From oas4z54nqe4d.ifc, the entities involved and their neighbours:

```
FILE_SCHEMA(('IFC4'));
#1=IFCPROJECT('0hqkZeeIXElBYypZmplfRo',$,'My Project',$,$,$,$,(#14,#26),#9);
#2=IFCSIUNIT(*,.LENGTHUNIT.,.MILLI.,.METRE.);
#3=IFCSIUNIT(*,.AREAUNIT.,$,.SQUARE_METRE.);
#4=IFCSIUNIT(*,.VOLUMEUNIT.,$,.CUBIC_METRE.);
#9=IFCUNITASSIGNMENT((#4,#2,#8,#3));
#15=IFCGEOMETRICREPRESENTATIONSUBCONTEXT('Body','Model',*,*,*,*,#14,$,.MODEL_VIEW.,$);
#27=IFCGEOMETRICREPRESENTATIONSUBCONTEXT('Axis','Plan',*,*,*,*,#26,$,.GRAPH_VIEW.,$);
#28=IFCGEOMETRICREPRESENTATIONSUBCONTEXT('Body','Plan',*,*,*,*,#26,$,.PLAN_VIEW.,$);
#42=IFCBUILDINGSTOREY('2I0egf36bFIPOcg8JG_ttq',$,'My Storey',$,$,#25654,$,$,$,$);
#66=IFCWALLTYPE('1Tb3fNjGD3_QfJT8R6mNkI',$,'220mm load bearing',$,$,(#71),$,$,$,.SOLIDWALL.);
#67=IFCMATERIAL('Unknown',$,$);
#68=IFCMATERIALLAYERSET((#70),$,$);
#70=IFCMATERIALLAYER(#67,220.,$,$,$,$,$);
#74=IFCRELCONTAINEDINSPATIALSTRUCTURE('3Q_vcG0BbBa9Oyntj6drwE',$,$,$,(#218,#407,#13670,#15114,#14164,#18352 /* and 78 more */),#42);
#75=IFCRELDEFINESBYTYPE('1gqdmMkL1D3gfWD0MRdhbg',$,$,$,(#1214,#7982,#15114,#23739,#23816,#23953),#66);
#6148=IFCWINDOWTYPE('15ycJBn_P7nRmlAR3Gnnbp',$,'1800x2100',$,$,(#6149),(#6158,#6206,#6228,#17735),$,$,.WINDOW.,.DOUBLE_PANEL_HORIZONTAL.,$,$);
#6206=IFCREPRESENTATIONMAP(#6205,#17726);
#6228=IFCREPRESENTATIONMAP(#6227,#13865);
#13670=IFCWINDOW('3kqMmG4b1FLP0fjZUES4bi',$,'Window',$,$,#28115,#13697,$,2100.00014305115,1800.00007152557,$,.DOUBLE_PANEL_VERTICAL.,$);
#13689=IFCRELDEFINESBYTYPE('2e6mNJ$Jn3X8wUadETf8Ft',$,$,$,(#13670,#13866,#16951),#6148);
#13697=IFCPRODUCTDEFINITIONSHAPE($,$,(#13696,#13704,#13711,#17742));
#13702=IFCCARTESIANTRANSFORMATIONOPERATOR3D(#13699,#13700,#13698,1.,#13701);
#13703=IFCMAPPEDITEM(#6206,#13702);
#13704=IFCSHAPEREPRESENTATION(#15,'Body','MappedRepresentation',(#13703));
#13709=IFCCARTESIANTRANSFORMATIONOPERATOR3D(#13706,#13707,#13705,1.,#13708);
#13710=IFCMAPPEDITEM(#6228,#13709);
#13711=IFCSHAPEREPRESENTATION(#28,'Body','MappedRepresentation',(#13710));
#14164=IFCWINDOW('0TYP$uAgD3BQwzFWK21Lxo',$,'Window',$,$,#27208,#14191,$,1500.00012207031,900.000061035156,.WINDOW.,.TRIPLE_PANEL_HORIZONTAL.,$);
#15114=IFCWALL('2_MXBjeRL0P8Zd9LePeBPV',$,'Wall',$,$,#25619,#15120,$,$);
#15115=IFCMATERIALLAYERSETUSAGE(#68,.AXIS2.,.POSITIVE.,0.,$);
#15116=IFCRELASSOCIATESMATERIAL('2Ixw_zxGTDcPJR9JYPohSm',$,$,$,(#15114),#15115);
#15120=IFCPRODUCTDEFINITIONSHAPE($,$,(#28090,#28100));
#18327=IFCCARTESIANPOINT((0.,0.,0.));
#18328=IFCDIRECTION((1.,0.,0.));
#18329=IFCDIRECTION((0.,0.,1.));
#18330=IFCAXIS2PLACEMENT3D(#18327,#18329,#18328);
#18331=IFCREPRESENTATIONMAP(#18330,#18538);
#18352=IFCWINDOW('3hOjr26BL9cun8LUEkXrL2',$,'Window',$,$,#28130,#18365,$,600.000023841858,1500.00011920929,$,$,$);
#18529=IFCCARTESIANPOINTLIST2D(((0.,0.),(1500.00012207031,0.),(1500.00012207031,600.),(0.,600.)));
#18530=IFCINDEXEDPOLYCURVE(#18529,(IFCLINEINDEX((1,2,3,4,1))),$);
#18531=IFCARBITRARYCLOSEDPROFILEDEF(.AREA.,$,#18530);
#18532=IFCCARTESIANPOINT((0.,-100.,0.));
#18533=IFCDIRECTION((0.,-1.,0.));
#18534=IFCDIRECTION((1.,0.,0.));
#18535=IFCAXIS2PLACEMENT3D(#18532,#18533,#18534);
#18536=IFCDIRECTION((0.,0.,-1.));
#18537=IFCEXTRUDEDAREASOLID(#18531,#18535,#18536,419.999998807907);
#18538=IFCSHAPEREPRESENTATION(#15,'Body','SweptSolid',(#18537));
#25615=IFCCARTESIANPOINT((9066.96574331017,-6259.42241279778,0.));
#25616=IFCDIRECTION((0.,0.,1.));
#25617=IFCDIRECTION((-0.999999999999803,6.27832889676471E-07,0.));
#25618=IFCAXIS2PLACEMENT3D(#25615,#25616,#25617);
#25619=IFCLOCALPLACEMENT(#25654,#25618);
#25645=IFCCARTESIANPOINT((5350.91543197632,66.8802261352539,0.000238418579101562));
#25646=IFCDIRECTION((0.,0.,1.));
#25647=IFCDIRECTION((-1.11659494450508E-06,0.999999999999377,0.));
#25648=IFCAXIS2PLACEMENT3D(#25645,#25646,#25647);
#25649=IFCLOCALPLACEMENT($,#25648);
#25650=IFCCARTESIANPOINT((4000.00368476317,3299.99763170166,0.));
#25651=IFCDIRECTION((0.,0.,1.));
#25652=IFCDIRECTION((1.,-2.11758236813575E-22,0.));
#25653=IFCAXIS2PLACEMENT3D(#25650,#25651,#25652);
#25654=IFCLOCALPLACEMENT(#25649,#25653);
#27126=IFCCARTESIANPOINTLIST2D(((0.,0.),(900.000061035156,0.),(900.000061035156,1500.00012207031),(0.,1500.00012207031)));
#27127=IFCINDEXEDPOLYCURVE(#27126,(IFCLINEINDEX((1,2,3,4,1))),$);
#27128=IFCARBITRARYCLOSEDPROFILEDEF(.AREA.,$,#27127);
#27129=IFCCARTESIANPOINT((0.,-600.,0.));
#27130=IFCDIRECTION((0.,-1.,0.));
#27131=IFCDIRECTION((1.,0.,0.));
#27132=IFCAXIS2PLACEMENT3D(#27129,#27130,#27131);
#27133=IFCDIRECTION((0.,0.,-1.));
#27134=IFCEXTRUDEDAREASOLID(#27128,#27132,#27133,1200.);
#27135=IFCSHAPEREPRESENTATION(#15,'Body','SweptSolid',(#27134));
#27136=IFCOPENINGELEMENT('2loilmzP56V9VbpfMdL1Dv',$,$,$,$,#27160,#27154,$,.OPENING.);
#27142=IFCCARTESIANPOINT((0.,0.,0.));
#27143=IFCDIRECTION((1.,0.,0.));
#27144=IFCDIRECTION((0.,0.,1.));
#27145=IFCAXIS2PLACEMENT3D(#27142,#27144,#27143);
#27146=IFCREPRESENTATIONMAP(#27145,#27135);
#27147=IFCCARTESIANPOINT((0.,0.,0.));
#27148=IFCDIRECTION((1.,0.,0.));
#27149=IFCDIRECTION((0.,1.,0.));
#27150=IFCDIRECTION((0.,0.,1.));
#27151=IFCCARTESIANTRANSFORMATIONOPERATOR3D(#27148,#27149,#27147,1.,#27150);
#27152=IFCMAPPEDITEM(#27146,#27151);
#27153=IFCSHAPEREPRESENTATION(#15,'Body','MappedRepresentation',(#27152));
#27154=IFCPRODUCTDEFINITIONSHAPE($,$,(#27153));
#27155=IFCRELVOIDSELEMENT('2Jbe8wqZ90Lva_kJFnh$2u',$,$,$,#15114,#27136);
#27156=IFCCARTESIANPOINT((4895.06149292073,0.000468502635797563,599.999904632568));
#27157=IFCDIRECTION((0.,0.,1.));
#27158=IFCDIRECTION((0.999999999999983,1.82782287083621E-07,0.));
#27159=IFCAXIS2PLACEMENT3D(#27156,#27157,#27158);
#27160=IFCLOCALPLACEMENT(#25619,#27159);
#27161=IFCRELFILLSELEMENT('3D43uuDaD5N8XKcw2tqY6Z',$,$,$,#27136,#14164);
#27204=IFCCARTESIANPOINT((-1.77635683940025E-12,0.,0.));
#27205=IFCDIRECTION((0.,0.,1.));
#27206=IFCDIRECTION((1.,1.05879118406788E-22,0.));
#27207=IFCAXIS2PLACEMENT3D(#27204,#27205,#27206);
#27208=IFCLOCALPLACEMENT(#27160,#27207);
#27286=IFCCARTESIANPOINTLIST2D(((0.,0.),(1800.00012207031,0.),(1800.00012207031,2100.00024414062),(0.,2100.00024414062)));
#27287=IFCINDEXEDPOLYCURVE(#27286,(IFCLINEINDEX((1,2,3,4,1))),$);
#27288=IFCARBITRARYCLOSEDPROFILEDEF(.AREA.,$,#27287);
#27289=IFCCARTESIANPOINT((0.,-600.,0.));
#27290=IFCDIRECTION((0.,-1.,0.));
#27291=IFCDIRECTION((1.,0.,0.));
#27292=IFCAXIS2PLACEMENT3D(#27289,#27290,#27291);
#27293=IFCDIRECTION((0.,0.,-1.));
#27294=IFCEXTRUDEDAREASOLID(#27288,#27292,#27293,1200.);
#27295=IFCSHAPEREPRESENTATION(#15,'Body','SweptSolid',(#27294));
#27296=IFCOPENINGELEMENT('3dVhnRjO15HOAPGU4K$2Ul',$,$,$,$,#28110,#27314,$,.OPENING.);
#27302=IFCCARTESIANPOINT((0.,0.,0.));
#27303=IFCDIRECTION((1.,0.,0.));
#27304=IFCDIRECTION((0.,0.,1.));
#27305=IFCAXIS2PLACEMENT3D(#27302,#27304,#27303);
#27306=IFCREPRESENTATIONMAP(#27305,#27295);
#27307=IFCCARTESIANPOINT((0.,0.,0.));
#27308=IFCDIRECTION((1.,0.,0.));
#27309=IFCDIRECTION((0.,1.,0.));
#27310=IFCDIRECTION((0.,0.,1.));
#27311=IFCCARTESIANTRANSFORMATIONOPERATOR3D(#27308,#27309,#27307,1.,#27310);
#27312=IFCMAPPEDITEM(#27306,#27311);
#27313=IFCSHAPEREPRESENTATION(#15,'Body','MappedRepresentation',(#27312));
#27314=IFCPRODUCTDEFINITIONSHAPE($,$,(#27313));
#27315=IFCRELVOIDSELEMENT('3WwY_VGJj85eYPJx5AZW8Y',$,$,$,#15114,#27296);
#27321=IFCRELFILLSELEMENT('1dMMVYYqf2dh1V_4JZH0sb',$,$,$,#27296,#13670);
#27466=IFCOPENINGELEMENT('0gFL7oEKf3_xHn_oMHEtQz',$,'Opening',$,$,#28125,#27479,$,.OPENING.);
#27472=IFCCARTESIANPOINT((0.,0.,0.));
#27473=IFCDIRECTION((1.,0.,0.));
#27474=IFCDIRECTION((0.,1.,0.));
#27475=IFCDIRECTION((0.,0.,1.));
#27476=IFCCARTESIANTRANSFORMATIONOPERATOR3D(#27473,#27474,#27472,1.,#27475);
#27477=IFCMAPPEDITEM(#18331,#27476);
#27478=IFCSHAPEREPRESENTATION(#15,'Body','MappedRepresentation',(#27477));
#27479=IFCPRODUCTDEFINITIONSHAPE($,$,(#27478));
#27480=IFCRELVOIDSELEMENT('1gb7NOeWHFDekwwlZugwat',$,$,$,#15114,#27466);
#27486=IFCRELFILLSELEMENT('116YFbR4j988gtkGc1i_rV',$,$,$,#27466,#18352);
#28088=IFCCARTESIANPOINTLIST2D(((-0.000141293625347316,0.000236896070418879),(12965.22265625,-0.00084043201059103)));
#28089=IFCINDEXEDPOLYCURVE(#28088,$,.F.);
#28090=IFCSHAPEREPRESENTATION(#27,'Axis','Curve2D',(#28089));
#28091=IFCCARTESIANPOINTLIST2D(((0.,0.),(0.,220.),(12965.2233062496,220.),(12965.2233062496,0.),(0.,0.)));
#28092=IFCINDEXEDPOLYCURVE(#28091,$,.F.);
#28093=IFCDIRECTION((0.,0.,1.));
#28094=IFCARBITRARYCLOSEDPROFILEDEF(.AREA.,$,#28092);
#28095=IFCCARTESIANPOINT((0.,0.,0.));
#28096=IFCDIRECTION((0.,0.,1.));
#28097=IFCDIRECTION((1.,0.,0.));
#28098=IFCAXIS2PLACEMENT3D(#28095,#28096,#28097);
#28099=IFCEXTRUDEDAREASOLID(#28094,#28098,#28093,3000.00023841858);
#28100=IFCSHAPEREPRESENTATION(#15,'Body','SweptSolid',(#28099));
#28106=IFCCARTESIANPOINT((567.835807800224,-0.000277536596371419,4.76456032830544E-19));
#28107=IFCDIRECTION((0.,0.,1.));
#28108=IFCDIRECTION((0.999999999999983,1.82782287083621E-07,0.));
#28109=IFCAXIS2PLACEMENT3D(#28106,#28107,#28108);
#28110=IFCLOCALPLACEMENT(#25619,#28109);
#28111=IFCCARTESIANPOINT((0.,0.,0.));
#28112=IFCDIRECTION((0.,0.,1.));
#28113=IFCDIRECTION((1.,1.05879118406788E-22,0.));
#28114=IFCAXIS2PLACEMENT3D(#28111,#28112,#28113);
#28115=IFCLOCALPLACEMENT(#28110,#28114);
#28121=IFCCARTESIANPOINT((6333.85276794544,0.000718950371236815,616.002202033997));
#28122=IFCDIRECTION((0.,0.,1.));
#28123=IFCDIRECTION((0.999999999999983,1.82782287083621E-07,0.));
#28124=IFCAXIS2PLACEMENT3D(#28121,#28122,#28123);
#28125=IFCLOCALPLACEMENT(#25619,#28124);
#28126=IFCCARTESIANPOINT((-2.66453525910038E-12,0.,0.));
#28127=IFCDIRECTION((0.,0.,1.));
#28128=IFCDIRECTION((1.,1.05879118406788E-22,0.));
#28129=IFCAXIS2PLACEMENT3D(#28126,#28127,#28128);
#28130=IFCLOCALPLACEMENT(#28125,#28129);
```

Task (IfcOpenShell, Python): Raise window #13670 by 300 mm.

```python
import numpy as np
import ifcopenshell
import ifcopenshell.api.geometry
import ifcopenshell.util.placement
import ifcopenshell.util.unit

model = ifcopenshell.open("oas4z54nqe4d.ifc")
unit_scale = ifcopenshell.util.unit.calculate_unit_scale(model)

window = model.by_guid("3kqMmG4b1FLP0fjZUES4bi")
opening = window.FillsVoids[0].RelatingOpeningElement
dz = 300.0

shift = np.array([0.0, 0.0, dz])
# The window is placed relative to its opening, so it follows when the opening moves.
matrix = ifcopenshell.util.placement.get_local_placement(opening.ObjectPlacement)
matrix[:3, 3] += shift
ifcopenshell.api.geometry.edit_object_placement(
    model, product=opening, matrix=matrix, is_si=False, should_transform_children=True
)

print(f"moved by {dz * unit_scale:+.3f} m")

model.write("oas4z54nqe4d_rev.ifc")
```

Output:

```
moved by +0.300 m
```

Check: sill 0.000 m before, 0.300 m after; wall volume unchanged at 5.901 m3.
